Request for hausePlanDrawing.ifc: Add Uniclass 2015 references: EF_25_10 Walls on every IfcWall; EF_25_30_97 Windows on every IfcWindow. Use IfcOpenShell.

First a look at what the model holds.

```python
import ifcopenshell

model = ifcopenshell.open("hausePlanDrawing.ifc")
print(model.schema)
print("classifications:", [c.Name for c in model.by_type("IfcClassification")])
for ifc_class in ("IfcDoor", "IfcRoof", "IfcStair", "IfcWall", "IfcWindow"):
    print(ifc_class, len(model.by_type(ifc_class)))
```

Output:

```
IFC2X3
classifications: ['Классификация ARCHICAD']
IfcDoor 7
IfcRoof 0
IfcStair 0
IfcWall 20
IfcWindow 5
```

```python
import ifcopenshell
import ifcopenshell.api.classification

model = ifcopenshell.open("hausePlanDrawing.ifc")

# IFC2X3 requires Source and Edition and has no link from the project to the system.
system = model.create_entity("IfcClassification", Source="NBS", Edition="2015", Name="Uniclass 2015")

codes = {
    "IfcWall": ("EF_25_10", "Walls"),
    "IfcWindow": ("EF_25_30_97", "Windows"),
}
for ifc_class, (code, name) in codes.items():
    products = model.by_type(ifc_class)
    ifcopenshell.api.classification.add_reference(
        model, products=products, classification=system, identification=code, name=name
    )
    print(code, len(products))

model.write("hausePlanDrawing_rev.ifc")
```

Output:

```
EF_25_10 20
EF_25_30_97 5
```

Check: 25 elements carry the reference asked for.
